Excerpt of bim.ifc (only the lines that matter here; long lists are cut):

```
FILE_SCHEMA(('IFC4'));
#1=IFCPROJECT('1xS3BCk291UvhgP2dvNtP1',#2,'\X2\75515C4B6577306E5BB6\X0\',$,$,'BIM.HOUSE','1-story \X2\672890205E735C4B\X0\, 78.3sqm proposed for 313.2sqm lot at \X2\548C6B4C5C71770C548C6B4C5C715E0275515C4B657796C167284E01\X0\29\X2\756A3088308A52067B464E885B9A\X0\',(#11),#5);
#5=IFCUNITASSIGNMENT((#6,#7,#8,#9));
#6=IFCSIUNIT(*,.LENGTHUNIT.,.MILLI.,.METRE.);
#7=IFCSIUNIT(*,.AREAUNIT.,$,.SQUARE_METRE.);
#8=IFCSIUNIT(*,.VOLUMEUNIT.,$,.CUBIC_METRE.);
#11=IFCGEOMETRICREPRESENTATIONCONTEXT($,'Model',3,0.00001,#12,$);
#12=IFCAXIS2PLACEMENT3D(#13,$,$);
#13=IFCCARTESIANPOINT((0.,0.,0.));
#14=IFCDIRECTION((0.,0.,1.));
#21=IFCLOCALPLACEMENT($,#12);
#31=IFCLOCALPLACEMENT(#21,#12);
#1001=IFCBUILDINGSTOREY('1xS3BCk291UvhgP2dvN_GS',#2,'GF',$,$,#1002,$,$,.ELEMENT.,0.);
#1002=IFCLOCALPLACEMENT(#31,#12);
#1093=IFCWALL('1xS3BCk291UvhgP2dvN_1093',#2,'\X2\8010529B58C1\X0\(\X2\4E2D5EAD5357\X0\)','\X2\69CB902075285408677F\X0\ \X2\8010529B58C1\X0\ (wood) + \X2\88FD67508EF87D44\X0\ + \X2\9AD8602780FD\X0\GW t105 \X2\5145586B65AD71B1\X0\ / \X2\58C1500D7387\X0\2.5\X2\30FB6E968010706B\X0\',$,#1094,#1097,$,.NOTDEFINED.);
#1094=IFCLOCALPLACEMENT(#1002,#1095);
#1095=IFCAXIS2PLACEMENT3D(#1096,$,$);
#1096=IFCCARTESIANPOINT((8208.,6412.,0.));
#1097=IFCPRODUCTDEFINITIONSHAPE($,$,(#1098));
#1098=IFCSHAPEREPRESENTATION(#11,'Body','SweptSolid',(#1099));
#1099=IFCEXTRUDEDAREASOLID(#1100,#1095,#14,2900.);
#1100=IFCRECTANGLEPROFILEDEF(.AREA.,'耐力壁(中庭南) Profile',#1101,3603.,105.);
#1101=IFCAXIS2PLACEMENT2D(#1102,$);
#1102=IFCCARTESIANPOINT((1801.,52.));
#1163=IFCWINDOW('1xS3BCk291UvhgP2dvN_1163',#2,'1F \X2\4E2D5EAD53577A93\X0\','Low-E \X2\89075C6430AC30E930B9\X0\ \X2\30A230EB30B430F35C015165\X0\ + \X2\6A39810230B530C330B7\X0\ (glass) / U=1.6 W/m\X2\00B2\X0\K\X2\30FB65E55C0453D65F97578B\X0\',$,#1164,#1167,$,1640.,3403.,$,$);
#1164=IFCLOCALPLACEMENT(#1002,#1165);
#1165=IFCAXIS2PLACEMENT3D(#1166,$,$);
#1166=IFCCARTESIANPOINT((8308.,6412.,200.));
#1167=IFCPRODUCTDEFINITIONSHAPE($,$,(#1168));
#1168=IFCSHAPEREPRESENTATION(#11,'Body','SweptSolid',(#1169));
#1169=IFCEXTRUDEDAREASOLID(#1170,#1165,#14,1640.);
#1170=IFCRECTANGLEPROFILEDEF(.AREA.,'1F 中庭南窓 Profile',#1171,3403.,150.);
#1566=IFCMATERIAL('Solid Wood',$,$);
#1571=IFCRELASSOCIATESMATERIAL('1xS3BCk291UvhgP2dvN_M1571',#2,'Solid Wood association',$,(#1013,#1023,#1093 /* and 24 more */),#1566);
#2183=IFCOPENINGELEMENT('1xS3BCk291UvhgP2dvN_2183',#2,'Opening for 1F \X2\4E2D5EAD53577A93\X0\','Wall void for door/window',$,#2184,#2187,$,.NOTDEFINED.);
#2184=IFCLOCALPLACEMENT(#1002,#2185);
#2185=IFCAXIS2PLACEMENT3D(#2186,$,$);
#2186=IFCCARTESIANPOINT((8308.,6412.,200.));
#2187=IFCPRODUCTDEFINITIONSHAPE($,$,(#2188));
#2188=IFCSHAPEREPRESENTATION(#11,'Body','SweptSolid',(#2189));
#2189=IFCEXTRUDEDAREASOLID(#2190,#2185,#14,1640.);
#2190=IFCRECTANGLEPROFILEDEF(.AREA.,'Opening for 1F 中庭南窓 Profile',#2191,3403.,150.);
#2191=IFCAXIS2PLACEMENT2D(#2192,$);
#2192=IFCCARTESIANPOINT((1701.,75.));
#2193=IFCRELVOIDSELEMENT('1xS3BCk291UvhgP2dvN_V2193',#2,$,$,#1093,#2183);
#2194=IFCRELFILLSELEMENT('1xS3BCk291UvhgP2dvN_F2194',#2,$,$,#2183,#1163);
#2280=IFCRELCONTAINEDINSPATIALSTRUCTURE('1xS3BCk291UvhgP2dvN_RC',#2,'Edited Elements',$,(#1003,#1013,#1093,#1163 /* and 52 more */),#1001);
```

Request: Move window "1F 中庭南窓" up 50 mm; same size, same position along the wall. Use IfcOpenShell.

```python
import numpy as np
import ifcopenshell
import ifcopenshell.api.geometry
import ifcopenshell.util.placement
import ifcopenshell.util.unit

model = ifcopenshell.open("bim.ifc")
unit_scale = ifcopenshell.util.unit.calculate_unit_scale(model)

window = model.by_guid("1xS3BCk291UvhgP2dvN_1163")
opening = window.FillsVoids[0].RelatingOpeningElement
dz = 50.0

shift = np.array([0.0, 0.0, dz])
# The window is not placed relative to its opening, so move both.
for product in (opening, window):
    matrix = ifcopenshell.util.placement.get_local_placement(product.ObjectPlacement)
    matrix[:3, 3] += shift
    ifcopenshell.api.geometry.edit_object_placement(model, product=product, matrix=matrix, is_si=False)

print(f"moved by {dz * unit_scale:+.3f} m")

model.write("bim_v2.ifc")
```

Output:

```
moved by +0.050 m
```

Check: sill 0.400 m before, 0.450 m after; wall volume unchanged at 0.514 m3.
